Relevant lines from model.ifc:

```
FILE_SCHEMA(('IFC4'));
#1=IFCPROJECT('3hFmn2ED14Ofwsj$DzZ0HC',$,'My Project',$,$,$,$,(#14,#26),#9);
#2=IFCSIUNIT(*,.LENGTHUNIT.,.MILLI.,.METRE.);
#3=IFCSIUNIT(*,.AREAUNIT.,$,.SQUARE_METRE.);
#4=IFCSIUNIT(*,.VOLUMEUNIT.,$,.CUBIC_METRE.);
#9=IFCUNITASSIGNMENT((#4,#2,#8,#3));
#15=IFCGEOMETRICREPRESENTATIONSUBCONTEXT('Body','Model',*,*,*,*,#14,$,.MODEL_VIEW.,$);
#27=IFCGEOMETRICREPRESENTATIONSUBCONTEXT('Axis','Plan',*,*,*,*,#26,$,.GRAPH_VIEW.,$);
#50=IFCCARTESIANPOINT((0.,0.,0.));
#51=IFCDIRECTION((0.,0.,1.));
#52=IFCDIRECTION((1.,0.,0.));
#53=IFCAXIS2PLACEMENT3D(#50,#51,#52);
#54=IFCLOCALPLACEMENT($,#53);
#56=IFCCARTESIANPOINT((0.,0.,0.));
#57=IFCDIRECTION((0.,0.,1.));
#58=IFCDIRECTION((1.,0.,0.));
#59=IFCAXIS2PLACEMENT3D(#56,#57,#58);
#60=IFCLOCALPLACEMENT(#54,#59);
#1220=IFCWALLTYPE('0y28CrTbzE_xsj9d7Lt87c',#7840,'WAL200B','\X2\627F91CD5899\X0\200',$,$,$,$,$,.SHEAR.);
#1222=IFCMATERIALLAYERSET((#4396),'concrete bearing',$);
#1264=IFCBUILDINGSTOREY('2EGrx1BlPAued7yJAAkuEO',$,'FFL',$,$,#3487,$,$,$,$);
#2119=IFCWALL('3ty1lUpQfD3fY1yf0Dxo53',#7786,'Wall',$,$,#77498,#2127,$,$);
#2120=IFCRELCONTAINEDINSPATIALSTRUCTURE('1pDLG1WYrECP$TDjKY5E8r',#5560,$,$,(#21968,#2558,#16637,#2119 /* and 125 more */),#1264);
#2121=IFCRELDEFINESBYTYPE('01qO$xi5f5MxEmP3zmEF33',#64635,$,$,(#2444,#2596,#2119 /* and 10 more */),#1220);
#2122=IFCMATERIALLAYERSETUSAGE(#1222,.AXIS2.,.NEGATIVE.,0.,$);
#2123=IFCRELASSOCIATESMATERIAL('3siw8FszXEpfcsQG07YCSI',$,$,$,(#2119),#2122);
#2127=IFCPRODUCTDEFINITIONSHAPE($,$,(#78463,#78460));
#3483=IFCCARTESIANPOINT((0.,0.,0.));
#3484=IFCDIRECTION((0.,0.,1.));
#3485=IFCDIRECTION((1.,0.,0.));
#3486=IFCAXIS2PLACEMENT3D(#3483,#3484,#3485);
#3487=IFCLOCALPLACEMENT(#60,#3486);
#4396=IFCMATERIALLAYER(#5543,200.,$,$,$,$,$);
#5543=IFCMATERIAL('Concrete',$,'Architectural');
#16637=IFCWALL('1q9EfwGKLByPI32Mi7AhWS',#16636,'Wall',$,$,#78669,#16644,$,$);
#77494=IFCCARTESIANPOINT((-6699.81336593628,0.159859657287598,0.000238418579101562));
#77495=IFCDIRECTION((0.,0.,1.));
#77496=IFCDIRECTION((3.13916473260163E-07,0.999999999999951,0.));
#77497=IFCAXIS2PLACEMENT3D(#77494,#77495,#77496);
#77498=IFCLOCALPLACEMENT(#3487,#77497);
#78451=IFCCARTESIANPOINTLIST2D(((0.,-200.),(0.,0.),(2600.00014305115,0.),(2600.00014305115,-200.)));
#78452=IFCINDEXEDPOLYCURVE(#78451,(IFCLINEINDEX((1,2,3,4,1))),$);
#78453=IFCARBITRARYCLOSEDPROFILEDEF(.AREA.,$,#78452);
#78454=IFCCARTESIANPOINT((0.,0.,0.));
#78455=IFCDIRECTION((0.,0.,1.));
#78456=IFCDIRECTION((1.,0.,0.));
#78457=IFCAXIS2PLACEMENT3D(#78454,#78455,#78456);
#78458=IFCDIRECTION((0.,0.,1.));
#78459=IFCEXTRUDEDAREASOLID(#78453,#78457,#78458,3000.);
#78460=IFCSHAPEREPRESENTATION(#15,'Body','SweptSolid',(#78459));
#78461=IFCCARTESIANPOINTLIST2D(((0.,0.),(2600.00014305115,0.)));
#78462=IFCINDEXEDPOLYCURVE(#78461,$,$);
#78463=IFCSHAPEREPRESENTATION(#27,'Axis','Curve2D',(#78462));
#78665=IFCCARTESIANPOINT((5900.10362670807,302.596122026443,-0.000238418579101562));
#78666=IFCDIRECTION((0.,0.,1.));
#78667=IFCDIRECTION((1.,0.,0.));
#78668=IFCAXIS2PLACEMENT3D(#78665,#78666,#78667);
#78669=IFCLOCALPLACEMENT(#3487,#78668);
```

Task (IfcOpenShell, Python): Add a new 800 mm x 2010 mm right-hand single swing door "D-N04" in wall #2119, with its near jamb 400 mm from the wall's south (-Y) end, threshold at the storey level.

```python
import numpy as np
import ifcopenshell
import ifcopenshell.api.feature
import ifcopenshell.api.geometry
import ifcopenshell.api.root
import ifcopenshell.api.spatial
import ifcopenshell.geom
import ifcopenshell.util.element
import ifcopenshell.util.placement
import ifcopenshell.util.representation
import ifcopenshell.util.shape
import ifcopenshell.util.unit

model = ifcopenshell.open("model.ifc")
unit_scale = ifcopenshell.util.unit.calculate_unit_scale(model)
settings = ifcopenshell.geom.settings()


def volume(element):
    """Net volume in cubic metres, openings subtracted."""
    shape = ifcopenshell.geom.create_shape(settings, element)
    return ifcopenshell.util.shape.get_volume(shape.geometry)


wall = model.by_guid("3ty1lUpQfD3fY1yf0Dxo53")
storey = ifcopenshell.util.element.get_container(wall, ifc_class="IfcBuildingStorey")
context = ifcopenshell.util.representation.get_context(model, "Model", "Body", "MODEL_VIEW")
before = volume(wall)

width, height, from_end, sill = 0.8, 2.01, 0.4, 0.0  # metres

# The wall runs along its own X axis, and the end named is its -X end.
wall_shape = ifcopenshell.geom.create_shape(settings, wall)
x, y, z = ifcopenshell.util.shape.get_vertices(wall_shape.geometry).T
start = x.min() + from_end
face, thickness = float(y.min()), float(y.max() - y.min())
wall_matrix = ifcopenshell.util.placement.get_local_placement(wall.ObjectPlacement)
level = ifcopenshell.util.placement.get_local_placement(storey.ObjectPlacement)[2, 3]


def in_wall(x, y):
    """Placement at x, y metres in the wall's axes, at sill height."""
    matrix = wall_matrix.copy()
    matrix[:, 3] = wall_matrix @ np.array([x / unit_scale, y / unit_scale, 0.0, 1.0])
    matrix[2, 3] = level + sill / unit_scale
    return matrix


# Opening: a box that overshoots both wall faces by 50 mm.
opening = ifcopenshell.api.root.create_entity(model, ifc_class="IfcOpeningElement", predefined_type="OPENING")
box = ifcopenshell.api.geometry.add_wall_representation(
    model, context=context, length=width, height=height, thickness=thickness + 0.1
)
ifcopenshell.api.geometry.assign_representation(model, product=opening, representation=box)
ifcopenshell.api.geometry.edit_object_placement(model, product=opening, matrix=in_wall(start, face - 0.05), is_si=False)
ifcopenshell.api.feature.add_feature(model, feature=opening, element=wall)

door = ifcopenshell.api.root.create_entity(model, ifc_class="IfcDoor", name="D-N04", predefined_type="DOOR")
door.OverallWidth, door.OverallHeight = width / unit_scale, height / unit_scale
door.OperationType = "SINGLE_SWING_RIGHT"
body = ifcopenshell.api.geometry.add_door_representation(
    model,
    context=context,
    overall_width=door.OverallWidth,
    overall_height=door.OverallHeight,
    operation_type="SINGLE_SWING_RIGHT",
    lining_properties={"LiningDepth": thickness / unit_scale, "ThresholdDepth": thickness / unit_scale},
)
ifcopenshell.api.geometry.assign_representation(model, product=door, representation=body)
ifcopenshell.api.spatial.assign_container(model, products=[door], relating_structure=storey)
ifcopenshell.api.feature.add_filling(model, opening=opening, element=door)

# The lining spans the wall, so the door starts at the wall face.
ifcopenshell.api.geometry.edit_object_placement(model, product=door, matrix=in_wall(start, face), is_si=False)

after = volume(wall)

print(f"wall volume {before:.3f} -> {after:.3f} m3")

model.write("model_v2.ifc")
```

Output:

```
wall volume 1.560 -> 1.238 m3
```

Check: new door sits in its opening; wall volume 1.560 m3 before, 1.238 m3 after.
